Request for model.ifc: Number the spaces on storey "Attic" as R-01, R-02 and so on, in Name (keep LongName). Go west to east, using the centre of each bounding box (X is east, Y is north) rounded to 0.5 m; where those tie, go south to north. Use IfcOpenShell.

First a look at what the model holds.

```python
import ifcopenshell
import ifcopenshell.util.element
import ifcopenshell.util.placement

model = ifcopenshell.open("model.ifc")
print(model.schema)
storey = next(s for s in model.by_type("IfcBuildingStorey") if s.Name == "Attic")
spaces = [e for e in ifcopenshell.util.element.get_decomposition(storey) if e.is_a("IfcSpace")]
for e in sorted(spaces, key=lambda e: e.id()):
    origin = ifcopenshell.util.placement.get_local_placement(e.ObjectPlacement)[:3, 3]
    print(e.id(), e.Name, e.LongName, origin.round(2) + 0.0, sep=" | ")
```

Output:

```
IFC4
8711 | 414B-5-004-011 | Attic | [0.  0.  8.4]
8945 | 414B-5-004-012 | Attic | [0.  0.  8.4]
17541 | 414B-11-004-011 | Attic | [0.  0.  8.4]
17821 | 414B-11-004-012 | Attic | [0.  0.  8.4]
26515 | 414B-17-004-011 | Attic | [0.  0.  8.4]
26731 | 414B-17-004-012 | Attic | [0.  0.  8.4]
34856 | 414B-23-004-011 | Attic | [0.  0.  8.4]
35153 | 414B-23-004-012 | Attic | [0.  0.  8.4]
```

```python
import ifcopenshell
import ifcopenshell.geom
import ifcopenshell.util.element
import ifcopenshell.util.shape

model = ifcopenshell.open("model.ifc")
settings = ifcopenshell.geom.settings()
settings.set("use-world-coords", True)


def centre(element):
    shape = ifcopenshell.geom.create_shape(settings, element)
    return ifcopenshell.util.shape.get_bbox_centroid(shape.geometry)


storey = next(s for s in model.by_type("IfcBuildingStorey") if s.Name == "Attic")
spaces = [e for e in ifcopenshell.util.element.get_decomposition(storey) if e.is_a("IfcSpace")]

# Insertion points can sit at a corner or the storey origin, so sort by the geometry (in metres).
centres = {e: centre(e) for e in spaces}
spaces.sort(key=lambda e: (round(centres[e][0] / 0.5), centres[e][1]))

for i, e in enumerate(spaces, start=1):
    number = f"R-{i:02d}"
    e.Name = number
    print(e.id(), number)

model.write("model_updated.ifc")
```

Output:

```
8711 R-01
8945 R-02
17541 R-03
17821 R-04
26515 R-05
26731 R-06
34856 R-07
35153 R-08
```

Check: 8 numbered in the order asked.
